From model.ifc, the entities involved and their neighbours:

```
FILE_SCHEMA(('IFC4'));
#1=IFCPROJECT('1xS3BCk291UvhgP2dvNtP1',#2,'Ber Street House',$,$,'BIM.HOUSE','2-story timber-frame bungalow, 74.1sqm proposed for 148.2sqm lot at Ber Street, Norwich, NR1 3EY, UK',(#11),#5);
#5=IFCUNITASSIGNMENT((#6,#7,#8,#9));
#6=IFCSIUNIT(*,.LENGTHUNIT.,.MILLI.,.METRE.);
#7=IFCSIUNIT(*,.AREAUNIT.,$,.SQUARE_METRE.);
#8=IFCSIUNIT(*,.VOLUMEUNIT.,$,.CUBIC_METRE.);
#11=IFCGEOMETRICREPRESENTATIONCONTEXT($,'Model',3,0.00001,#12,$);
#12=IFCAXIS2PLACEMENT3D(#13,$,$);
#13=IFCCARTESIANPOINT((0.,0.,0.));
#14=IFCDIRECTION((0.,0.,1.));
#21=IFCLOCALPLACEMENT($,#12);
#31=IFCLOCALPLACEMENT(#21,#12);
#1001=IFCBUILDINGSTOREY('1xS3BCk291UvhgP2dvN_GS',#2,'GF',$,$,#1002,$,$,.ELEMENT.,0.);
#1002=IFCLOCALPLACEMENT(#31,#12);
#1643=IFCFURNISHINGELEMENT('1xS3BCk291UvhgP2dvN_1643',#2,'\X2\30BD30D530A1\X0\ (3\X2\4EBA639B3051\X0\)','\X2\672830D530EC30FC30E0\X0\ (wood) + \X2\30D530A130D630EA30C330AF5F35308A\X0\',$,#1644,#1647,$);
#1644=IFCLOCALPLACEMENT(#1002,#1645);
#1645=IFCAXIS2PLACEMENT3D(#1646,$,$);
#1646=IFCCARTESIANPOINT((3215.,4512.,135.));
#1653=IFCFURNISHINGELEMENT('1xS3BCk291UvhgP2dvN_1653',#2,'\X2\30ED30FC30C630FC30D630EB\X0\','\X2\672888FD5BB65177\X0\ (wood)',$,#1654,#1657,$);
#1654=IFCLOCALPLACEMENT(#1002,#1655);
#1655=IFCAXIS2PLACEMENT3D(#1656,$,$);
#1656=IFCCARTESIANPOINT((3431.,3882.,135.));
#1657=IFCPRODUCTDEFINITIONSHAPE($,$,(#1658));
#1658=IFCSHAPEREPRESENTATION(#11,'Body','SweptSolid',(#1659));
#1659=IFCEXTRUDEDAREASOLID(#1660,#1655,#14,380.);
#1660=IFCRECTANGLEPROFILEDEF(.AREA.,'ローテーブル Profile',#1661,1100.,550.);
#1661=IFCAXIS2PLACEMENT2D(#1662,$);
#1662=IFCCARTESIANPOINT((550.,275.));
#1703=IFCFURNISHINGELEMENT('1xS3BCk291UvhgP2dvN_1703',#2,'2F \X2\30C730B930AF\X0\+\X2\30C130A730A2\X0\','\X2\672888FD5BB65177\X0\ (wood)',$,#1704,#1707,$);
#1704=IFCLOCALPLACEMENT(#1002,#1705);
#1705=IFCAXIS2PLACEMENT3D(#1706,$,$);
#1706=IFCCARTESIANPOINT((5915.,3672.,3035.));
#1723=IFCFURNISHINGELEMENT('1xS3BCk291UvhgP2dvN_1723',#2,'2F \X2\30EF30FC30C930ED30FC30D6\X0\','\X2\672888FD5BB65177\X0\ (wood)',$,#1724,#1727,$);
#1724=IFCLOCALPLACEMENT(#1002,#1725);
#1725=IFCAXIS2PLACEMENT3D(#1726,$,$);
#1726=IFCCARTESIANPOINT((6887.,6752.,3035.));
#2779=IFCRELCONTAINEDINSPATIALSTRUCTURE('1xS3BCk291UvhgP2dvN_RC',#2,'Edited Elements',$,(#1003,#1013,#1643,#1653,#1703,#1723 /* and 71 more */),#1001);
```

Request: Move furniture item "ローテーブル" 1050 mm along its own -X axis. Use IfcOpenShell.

```python
import ifcopenshell
import ifcopenshell.api.geometry
import ifcopenshell.util.placement

model = ifcopenshell.open("model.ifc")

item = model.by_guid("1xS3BCk291UvhgP2dvN_1653")
matrix = ifcopenshell.util.placement.get_local_placement(item.ObjectPlacement)
matrix[:3, 3] -= matrix[:3, 0] * 1050.0
ifcopenshell.api.geometry.edit_object_placement(model, product=item, matrix=matrix, is_si=False)

print(ifcopenshell.util.placement.get_local_placement(item.ObjectPlacement).round(3) + 0.0)

model.write("model_updated.ifc")
```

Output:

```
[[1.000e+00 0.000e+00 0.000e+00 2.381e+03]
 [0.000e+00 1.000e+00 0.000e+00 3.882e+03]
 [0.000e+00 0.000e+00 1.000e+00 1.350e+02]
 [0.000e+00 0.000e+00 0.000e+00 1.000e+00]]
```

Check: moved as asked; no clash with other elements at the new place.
